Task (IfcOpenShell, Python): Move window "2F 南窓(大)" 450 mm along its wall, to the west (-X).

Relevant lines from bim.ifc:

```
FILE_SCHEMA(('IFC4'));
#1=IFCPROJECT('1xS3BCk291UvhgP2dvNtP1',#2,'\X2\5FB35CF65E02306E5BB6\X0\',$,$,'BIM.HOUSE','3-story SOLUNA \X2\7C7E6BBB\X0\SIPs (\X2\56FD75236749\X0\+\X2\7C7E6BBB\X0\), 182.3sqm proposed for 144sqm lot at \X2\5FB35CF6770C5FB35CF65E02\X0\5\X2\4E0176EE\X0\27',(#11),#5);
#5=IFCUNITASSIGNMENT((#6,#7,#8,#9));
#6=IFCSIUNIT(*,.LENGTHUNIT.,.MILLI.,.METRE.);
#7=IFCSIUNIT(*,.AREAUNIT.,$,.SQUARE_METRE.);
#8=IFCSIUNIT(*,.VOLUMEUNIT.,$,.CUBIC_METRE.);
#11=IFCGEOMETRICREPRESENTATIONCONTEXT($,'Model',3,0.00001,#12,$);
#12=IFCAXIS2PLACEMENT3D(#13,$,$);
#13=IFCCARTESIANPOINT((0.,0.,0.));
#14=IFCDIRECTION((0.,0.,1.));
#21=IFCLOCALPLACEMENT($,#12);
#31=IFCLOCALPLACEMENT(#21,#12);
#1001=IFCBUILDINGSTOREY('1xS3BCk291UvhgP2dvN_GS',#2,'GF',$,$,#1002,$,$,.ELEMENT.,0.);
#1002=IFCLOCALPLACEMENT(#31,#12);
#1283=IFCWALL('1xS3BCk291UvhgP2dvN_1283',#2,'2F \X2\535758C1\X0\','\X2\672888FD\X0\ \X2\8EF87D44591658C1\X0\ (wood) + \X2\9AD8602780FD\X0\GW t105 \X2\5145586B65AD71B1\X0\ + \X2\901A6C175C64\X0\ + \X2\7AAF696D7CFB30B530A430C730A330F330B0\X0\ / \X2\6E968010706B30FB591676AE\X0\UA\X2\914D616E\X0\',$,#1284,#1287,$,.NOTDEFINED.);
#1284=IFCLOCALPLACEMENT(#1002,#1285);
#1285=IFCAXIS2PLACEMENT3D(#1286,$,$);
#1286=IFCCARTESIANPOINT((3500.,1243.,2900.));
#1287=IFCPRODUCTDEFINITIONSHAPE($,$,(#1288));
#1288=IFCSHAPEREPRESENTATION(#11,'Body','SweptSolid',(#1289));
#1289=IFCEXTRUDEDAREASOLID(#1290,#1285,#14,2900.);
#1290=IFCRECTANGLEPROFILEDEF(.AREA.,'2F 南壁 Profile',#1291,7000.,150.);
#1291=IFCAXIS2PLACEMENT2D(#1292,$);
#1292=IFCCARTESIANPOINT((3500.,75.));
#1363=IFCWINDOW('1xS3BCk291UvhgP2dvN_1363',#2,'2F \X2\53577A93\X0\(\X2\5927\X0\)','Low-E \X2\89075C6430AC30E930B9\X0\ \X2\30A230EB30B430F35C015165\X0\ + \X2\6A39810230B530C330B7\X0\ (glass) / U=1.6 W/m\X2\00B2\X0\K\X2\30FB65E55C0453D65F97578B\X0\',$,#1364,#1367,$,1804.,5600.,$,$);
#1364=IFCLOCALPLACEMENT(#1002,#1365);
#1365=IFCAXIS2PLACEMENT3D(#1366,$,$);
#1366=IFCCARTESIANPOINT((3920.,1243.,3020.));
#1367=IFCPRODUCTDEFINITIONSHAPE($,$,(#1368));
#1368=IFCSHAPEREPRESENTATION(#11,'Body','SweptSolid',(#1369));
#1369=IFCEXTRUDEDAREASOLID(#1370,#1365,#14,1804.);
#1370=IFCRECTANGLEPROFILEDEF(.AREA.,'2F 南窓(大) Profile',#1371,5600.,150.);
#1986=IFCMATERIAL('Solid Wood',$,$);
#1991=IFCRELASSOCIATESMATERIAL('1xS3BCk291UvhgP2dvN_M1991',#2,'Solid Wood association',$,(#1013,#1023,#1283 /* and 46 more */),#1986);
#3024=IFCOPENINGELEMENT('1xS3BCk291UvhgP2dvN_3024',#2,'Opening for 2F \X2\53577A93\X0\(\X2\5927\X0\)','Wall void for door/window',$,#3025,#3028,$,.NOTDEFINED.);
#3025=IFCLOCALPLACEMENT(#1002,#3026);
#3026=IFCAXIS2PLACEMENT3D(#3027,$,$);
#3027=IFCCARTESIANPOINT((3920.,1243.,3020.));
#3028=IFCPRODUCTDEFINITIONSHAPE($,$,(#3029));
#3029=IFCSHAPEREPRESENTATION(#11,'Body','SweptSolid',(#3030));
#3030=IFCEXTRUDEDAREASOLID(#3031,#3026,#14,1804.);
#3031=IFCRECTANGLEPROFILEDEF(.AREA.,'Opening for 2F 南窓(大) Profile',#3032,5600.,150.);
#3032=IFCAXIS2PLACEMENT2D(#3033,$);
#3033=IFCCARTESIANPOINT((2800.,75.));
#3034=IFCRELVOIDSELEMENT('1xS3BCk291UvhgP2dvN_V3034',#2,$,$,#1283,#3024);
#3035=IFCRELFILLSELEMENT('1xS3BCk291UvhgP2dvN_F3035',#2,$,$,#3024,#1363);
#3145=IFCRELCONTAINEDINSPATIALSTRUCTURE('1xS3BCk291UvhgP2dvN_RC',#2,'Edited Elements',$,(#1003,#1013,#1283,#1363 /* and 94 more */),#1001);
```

```python
import ifcopenshell
import ifcopenshell.api.geometry
import ifcopenshell.util.placement
import ifcopenshell.util.unit

model = ifcopenshell.open("bim.ifc")
unit_scale = ifcopenshell.util.unit.calculate_unit_scale(model)

window = model.by_id(1363)
opening = window.FillsVoids[0].RelatingOpeningElement
wall = opening.VoidsElements[0].RelatingBuildingElement

wall_matrix = ifcopenshell.util.placement.get_local_placement(wall.ObjectPlacement)
shift = wall_matrix[:3, 0] * -0.45 / unit_scale
before = ifcopenshell.util.placement.get_local_placement(window.ObjectPlacement)[:3, 3].copy()

# The window is not placed relative to its opening, so move both.
for product in (opening, window):
    matrix = ifcopenshell.util.placement.get_local_placement(product.ObjectPlacement)
    matrix[:3, 3] += shift
    ifcopenshell.api.geometry.edit_object_placement(model, product=product, matrix=matrix, is_si=False)

after = ifcopenshell.util.placement.get_local_placement(window.ObjectPlacement)[:3, 3]
print("window moved by", (after - before).round(3) + 0.0)

model.write("bim_v2.ifc")
```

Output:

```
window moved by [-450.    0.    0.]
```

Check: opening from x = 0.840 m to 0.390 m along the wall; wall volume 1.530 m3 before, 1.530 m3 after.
